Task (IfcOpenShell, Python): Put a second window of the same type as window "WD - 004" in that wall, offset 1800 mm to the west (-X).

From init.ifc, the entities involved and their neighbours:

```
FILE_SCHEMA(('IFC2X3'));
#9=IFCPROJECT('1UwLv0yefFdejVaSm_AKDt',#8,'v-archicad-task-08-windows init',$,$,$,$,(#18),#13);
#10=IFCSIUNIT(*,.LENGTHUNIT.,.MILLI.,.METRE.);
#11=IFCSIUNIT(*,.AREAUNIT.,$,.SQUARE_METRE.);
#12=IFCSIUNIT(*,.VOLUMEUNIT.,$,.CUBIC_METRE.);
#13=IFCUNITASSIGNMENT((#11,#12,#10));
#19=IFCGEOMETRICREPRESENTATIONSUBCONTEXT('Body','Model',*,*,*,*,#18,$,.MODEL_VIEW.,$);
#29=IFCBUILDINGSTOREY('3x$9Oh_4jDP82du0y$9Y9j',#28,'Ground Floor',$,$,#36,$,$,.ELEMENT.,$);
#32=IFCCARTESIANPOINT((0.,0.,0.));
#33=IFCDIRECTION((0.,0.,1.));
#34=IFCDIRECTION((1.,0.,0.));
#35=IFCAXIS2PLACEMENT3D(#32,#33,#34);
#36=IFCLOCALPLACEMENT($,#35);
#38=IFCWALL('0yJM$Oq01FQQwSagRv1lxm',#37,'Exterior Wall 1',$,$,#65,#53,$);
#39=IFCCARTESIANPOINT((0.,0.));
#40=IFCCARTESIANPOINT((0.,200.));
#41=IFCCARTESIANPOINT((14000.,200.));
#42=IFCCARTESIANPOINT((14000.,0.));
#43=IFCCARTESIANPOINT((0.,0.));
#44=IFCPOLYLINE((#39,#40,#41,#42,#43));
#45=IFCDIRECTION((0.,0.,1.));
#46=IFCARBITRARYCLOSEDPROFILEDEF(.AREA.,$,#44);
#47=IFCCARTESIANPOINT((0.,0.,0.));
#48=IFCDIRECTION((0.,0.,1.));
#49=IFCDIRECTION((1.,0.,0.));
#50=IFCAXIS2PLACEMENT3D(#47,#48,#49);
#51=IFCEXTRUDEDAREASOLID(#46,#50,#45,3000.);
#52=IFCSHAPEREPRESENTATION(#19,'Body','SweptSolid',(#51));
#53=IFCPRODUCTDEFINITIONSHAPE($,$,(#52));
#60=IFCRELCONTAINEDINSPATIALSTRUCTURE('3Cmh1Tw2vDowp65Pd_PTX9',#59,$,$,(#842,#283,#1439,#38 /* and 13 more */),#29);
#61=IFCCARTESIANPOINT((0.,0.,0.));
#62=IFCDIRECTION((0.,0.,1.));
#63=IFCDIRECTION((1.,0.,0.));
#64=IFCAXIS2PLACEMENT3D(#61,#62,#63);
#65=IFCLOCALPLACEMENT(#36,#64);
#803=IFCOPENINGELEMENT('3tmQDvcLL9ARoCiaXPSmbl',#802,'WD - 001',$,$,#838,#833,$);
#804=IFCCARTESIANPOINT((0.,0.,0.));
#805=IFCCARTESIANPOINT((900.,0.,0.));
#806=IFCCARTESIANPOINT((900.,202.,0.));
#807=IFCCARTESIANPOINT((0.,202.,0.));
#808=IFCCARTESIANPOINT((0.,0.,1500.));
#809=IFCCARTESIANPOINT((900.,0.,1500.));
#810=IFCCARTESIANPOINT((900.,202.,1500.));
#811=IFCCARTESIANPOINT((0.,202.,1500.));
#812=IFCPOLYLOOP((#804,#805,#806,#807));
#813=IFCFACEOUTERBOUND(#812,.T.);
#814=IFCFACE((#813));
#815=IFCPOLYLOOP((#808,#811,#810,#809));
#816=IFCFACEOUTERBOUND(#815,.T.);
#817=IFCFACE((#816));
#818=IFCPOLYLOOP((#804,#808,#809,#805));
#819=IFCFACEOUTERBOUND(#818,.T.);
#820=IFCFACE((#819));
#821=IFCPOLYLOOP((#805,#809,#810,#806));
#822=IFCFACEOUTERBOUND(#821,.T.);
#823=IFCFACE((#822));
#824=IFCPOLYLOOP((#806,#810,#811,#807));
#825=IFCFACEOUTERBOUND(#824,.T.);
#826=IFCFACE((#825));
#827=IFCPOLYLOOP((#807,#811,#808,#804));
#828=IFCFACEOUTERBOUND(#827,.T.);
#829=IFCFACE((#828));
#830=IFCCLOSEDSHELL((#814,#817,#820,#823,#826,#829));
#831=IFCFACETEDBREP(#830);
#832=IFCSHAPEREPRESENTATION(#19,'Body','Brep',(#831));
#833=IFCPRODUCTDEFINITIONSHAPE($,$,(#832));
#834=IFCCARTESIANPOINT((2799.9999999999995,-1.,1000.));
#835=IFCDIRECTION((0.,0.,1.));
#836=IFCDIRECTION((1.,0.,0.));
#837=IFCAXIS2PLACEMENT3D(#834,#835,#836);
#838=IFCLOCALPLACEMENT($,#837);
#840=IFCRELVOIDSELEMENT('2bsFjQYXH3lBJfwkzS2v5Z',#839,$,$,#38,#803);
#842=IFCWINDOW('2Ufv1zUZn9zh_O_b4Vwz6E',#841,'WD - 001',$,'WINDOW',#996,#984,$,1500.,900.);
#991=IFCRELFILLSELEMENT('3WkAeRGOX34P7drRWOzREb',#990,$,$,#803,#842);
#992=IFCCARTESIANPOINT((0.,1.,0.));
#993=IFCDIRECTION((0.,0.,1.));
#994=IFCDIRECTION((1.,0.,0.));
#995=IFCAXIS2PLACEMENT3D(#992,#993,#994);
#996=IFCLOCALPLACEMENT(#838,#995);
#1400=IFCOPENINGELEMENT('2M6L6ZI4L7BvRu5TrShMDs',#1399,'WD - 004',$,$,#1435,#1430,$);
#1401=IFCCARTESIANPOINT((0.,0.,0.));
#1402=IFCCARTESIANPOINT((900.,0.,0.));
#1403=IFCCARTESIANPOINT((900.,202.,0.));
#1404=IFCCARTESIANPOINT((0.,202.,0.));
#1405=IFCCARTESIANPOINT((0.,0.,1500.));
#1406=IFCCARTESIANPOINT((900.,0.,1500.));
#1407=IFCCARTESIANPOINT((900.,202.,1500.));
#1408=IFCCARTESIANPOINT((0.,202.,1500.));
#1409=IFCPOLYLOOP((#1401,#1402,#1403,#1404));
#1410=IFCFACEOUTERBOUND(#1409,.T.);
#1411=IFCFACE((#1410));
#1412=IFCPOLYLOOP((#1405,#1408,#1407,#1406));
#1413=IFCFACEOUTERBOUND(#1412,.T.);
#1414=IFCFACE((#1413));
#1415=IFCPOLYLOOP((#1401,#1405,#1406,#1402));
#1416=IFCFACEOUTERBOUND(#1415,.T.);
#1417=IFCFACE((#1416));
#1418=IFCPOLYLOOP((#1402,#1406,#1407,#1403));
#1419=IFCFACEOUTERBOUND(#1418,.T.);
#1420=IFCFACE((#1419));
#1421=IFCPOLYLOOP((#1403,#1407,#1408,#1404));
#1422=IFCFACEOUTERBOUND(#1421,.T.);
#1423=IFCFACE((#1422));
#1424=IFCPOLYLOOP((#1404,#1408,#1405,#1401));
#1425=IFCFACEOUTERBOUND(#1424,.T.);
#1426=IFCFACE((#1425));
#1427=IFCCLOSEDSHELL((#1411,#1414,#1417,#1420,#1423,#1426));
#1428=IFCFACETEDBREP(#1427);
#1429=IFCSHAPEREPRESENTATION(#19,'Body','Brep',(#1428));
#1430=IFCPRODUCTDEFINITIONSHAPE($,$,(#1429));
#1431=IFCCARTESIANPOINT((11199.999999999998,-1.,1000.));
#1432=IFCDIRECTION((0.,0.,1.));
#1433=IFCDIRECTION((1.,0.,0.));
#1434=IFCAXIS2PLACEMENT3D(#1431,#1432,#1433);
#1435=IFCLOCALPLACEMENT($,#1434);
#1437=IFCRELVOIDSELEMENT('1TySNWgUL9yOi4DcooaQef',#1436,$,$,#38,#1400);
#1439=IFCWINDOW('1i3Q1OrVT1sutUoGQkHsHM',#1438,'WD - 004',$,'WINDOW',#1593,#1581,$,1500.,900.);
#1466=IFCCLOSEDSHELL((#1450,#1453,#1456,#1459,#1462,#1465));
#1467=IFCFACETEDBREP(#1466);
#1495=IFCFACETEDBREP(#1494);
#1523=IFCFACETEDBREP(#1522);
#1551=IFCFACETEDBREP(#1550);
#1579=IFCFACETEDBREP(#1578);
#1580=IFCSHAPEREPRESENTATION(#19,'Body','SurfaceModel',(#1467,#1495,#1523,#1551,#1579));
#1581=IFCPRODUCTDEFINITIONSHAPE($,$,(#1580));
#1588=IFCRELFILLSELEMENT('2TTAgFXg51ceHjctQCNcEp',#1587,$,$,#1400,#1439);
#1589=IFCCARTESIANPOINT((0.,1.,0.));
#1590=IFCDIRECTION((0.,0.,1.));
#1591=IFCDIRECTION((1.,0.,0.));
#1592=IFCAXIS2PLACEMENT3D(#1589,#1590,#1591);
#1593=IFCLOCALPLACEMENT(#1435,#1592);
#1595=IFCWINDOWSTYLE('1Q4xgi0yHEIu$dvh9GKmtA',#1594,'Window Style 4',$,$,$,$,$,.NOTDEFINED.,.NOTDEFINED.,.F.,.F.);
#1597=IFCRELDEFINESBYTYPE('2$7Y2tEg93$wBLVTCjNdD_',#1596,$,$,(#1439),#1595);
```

```python
import ifcopenshell
import ifcopenshell.api.feature
import ifcopenshell.api.geometry
import ifcopenshell.api.root
import ifcopenshell.geom
import ifcopenshell.util.element
import ifcopenshell.util.placement
import ifcopenshell.util.shape

model = ifcopenshell.open("init.ifc")
settings = ifcopenshell.geom.settings()


def volume(element):
    """Net volume in cubic metres, openings subtracted."""
    shape = ifcopenshell.geom.create_shape(settings, element)
    return ifcopenshell.util.shape.get_volume(shape.geometry)


window = model.by_guid("1i3Q1OrVT1sutUoGQkHsHM")
opening = window.FillsVoids[0].RelatingOpeningElement
wall = opening.VoidsElements[0].RelatingBuildingElement
before = volume(wall)
shift = ifcopenshell.util.placement.get_local_placement(wall.ObjectPlacement)[:3, 0] * -1800.0

# copy_class copies the void relationship, type, container and properties, but no geometry.
new_opening = ifcopenshell.api.root.copy_class(model, product=opening)
new_opening.Representation = ifcopenshell.util.element.copy_deep(
    model, opening.Representation, exclude=["IfcGeometricRepresentationContext", "IfcRepresentationMap"]
)
new_window = ifcopenshell.api.root.copy_class(model, product=window)
new_window.Representation = ifcopenshell.util.element.copy_deep(
    model, window.Representation, exclude=["IfcGeometricRepresentationContext", "IfcRepresentationMap"]
)
fills = ifcopenshell.api.feature.add_filling(model, opening=new_opening, element=new_window)
fills.OwnerHistory = new_window.OwnerHistory  # required in IFC2X3

for old, new in ((opening, new_opening), (window, new_window)):
    matrix = ifcopenshell.util.placement.get_local_placement(old.ObjectPlacement)
    matrix[:3, 3] += shift
    ifcopenshell.api.geometry.edit_object_placement(model, product=new, matrix=matrix, is_si=False)

after = volume(wall)

print(f"wall volume {before:.3f} -> {after:.3f} m3")

model.write("init_edited.ifc")
```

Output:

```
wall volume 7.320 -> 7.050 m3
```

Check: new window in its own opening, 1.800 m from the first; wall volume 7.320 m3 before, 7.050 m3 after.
